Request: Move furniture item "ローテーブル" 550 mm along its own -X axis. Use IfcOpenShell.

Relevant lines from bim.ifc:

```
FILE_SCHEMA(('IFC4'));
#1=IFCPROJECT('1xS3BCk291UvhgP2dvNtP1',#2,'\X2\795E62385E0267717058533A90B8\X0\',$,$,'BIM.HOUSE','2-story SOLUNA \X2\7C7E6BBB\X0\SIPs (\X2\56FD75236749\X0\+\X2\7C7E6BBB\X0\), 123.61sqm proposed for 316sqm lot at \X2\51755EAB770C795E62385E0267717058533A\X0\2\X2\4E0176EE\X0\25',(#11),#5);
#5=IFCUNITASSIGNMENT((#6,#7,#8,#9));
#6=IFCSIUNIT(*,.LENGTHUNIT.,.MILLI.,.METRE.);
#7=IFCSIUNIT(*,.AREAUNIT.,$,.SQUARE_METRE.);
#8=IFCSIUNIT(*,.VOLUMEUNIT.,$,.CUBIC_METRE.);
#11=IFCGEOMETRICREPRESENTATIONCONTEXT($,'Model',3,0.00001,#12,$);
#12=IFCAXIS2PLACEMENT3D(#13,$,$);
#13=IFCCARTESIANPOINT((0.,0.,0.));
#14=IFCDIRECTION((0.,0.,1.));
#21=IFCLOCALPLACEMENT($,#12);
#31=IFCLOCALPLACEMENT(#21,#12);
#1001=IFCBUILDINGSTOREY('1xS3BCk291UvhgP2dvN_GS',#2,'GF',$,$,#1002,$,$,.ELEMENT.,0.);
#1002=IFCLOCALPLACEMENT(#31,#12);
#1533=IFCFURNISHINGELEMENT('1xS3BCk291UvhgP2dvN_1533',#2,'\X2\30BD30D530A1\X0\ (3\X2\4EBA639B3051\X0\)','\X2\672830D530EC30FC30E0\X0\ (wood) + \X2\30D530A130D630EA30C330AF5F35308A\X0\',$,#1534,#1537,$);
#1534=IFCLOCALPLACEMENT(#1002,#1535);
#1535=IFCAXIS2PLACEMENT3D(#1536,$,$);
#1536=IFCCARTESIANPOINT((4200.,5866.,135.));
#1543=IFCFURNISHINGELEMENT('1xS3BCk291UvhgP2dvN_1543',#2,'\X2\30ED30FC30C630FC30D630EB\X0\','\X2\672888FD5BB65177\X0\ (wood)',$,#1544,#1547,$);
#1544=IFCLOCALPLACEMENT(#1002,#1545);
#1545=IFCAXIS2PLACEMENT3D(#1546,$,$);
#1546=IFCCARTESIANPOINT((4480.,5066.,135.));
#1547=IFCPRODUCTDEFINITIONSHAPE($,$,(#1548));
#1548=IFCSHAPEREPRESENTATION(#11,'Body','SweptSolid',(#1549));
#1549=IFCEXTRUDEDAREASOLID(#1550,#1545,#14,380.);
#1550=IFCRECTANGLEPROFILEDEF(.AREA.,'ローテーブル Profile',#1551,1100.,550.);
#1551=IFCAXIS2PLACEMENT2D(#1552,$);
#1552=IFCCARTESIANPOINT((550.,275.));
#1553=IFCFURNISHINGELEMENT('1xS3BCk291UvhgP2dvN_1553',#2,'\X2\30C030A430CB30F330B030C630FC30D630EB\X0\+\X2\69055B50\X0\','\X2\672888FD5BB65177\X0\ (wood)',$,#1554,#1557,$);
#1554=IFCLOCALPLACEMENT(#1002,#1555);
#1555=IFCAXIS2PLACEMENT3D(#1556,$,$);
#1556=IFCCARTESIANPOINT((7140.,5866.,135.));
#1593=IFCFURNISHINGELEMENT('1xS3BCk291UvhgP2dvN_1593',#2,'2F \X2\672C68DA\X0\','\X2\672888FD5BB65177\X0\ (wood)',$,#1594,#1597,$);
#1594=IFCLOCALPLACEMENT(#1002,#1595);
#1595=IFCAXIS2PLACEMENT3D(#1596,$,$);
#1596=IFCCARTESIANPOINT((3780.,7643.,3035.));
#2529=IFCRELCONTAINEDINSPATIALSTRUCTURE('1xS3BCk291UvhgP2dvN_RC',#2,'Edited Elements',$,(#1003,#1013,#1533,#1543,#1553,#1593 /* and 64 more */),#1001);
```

```python
import ifcopenshell
import ifcopenshell.api.geometry
import ifcopenshell.util.placement

model = ifcopenshell.open("bim.ifc")

item = model.by_guid("1xS3BCk291UvhgP2dvN_1543")
matrix = ifcopenshell.util.placement.get_local_placement(item.ObjectPlacement)
matrix[:3, 3] -= matrix[:3, 0] * 550.0
ifcopenshell.api.geometry.edit_object_placement(model, product=item, matrix=matrix, is_si=False)

print(ifcopenshell.util.placement.get_local_placement(item.ObjectPlacement).round(3) + 0.0)

model.write("bim_updated.ifc")
```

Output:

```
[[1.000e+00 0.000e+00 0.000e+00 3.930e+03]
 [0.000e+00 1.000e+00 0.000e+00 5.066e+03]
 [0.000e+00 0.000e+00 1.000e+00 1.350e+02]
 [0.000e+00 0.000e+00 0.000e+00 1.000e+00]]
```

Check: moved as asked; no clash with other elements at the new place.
